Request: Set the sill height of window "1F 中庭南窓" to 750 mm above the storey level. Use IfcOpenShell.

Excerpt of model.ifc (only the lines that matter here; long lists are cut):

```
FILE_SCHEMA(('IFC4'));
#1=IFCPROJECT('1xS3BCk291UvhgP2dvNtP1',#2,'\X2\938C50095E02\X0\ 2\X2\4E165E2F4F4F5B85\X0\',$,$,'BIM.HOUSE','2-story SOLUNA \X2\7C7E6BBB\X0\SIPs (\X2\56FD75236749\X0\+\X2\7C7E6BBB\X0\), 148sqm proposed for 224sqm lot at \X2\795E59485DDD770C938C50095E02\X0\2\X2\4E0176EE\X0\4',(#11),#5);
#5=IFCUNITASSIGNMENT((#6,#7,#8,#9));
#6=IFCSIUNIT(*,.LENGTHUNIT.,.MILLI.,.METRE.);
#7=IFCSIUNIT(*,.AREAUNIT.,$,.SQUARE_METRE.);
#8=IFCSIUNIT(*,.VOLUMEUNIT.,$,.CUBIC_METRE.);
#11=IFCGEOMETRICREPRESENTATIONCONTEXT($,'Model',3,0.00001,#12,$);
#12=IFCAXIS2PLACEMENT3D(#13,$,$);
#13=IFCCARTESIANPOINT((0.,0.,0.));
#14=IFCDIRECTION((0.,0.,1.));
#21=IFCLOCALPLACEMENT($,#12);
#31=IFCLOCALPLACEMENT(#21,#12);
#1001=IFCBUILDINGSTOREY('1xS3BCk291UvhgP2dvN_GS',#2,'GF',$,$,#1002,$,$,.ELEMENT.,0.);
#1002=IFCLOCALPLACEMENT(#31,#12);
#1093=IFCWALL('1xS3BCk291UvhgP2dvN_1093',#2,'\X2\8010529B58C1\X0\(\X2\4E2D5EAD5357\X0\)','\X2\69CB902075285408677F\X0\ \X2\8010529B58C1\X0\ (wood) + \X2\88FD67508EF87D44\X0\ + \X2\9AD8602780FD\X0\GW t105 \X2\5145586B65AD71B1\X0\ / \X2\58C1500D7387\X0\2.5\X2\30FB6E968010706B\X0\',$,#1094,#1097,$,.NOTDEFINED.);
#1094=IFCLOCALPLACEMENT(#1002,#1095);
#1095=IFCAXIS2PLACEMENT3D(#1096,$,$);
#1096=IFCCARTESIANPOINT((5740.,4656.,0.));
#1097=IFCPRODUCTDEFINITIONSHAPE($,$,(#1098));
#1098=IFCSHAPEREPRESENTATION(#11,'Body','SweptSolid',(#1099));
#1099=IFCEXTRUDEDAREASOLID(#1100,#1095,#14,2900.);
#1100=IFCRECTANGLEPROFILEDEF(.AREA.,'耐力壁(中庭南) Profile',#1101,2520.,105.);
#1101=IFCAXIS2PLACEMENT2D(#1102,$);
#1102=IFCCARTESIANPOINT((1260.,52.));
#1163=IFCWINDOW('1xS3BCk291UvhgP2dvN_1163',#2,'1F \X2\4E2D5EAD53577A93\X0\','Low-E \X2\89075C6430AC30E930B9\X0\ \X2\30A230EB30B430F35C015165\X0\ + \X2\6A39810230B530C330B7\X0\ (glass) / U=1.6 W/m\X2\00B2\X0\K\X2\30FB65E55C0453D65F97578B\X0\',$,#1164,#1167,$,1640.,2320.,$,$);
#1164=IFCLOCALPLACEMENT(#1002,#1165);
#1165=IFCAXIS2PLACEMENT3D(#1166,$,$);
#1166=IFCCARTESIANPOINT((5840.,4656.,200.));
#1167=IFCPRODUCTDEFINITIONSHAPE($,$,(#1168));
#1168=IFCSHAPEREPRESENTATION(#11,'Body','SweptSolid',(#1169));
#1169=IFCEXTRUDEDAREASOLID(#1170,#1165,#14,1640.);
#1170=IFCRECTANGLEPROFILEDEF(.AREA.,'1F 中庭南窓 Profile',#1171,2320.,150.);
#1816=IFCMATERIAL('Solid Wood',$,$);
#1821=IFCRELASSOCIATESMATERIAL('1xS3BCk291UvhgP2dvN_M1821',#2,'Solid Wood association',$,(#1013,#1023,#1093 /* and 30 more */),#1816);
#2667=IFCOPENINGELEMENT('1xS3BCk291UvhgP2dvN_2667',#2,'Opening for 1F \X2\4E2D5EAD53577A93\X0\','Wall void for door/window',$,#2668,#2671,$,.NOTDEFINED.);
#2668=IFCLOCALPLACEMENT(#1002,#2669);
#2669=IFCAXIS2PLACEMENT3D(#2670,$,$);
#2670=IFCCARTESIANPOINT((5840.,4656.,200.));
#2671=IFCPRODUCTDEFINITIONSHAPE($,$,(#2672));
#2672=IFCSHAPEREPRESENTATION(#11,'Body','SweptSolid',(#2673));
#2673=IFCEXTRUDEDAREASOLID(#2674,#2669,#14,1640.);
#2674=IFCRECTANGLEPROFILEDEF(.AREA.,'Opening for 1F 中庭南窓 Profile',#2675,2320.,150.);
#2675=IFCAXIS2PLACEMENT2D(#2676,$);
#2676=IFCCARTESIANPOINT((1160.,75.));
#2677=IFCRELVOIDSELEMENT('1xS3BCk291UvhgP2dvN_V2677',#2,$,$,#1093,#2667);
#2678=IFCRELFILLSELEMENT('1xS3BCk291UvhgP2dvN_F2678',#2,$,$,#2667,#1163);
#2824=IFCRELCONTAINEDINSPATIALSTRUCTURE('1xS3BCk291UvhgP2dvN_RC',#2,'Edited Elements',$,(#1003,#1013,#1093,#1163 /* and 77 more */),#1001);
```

```python
import numpy as np
import ifcopenshell
import ifcopenshell.api.geometry
import ifcopenshell.geom
import ifcopenshell.util.element
import ifcopenshell.util.placement
import ifcopenshell.util.shape
import ifcopenshell.util.unit

model = ifcopenshell.open("model.ifc")
unit_scale = ifcopenshell.util.unit.calculate_unit_scale(model)

window = model.by_guid("1xS3BCk291UvhgP2dvN_1163")
opening = window.FillsVoids[0].RelatingOpeningElement
storey = ifcopenshell.util.element.get_container(window, ifc_class="IfcBuildingStorey")
level = ifcopenshell.util.placement.get_local_placement(storey.ObjectPlacement)[2, 3]

# The opening's origin need not be at the sill, so measure its lowest point.
shape = ifcopenshell.geom.create_shape(ifcopenshell.geom.settings(), opening)
bottom = ifcopenshell.util.shape.get_shape_bottom_elevation(shape, shape.geometry) / unit_scale
dz = level + 0.75 / unit_scale - bottom

shift = np.array([0.0, 0.0, dz])
# The window is not placed relative to its opening, so move both.
for product in (opening, window):
    matrix = ifcopenshell.util.placement.get_local_placement(product.ObjectPlacement)
    matrix[:3, 3] += shift
    ifcopenshell.api.geometry.edit_object_placement(model, product=product, matrix=matrix, is_si=False)

print(f"moved by {dz * unit_scale:+.3f} m")

model.write("model-out.ifc")
```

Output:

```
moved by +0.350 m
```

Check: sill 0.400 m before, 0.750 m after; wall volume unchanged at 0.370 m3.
